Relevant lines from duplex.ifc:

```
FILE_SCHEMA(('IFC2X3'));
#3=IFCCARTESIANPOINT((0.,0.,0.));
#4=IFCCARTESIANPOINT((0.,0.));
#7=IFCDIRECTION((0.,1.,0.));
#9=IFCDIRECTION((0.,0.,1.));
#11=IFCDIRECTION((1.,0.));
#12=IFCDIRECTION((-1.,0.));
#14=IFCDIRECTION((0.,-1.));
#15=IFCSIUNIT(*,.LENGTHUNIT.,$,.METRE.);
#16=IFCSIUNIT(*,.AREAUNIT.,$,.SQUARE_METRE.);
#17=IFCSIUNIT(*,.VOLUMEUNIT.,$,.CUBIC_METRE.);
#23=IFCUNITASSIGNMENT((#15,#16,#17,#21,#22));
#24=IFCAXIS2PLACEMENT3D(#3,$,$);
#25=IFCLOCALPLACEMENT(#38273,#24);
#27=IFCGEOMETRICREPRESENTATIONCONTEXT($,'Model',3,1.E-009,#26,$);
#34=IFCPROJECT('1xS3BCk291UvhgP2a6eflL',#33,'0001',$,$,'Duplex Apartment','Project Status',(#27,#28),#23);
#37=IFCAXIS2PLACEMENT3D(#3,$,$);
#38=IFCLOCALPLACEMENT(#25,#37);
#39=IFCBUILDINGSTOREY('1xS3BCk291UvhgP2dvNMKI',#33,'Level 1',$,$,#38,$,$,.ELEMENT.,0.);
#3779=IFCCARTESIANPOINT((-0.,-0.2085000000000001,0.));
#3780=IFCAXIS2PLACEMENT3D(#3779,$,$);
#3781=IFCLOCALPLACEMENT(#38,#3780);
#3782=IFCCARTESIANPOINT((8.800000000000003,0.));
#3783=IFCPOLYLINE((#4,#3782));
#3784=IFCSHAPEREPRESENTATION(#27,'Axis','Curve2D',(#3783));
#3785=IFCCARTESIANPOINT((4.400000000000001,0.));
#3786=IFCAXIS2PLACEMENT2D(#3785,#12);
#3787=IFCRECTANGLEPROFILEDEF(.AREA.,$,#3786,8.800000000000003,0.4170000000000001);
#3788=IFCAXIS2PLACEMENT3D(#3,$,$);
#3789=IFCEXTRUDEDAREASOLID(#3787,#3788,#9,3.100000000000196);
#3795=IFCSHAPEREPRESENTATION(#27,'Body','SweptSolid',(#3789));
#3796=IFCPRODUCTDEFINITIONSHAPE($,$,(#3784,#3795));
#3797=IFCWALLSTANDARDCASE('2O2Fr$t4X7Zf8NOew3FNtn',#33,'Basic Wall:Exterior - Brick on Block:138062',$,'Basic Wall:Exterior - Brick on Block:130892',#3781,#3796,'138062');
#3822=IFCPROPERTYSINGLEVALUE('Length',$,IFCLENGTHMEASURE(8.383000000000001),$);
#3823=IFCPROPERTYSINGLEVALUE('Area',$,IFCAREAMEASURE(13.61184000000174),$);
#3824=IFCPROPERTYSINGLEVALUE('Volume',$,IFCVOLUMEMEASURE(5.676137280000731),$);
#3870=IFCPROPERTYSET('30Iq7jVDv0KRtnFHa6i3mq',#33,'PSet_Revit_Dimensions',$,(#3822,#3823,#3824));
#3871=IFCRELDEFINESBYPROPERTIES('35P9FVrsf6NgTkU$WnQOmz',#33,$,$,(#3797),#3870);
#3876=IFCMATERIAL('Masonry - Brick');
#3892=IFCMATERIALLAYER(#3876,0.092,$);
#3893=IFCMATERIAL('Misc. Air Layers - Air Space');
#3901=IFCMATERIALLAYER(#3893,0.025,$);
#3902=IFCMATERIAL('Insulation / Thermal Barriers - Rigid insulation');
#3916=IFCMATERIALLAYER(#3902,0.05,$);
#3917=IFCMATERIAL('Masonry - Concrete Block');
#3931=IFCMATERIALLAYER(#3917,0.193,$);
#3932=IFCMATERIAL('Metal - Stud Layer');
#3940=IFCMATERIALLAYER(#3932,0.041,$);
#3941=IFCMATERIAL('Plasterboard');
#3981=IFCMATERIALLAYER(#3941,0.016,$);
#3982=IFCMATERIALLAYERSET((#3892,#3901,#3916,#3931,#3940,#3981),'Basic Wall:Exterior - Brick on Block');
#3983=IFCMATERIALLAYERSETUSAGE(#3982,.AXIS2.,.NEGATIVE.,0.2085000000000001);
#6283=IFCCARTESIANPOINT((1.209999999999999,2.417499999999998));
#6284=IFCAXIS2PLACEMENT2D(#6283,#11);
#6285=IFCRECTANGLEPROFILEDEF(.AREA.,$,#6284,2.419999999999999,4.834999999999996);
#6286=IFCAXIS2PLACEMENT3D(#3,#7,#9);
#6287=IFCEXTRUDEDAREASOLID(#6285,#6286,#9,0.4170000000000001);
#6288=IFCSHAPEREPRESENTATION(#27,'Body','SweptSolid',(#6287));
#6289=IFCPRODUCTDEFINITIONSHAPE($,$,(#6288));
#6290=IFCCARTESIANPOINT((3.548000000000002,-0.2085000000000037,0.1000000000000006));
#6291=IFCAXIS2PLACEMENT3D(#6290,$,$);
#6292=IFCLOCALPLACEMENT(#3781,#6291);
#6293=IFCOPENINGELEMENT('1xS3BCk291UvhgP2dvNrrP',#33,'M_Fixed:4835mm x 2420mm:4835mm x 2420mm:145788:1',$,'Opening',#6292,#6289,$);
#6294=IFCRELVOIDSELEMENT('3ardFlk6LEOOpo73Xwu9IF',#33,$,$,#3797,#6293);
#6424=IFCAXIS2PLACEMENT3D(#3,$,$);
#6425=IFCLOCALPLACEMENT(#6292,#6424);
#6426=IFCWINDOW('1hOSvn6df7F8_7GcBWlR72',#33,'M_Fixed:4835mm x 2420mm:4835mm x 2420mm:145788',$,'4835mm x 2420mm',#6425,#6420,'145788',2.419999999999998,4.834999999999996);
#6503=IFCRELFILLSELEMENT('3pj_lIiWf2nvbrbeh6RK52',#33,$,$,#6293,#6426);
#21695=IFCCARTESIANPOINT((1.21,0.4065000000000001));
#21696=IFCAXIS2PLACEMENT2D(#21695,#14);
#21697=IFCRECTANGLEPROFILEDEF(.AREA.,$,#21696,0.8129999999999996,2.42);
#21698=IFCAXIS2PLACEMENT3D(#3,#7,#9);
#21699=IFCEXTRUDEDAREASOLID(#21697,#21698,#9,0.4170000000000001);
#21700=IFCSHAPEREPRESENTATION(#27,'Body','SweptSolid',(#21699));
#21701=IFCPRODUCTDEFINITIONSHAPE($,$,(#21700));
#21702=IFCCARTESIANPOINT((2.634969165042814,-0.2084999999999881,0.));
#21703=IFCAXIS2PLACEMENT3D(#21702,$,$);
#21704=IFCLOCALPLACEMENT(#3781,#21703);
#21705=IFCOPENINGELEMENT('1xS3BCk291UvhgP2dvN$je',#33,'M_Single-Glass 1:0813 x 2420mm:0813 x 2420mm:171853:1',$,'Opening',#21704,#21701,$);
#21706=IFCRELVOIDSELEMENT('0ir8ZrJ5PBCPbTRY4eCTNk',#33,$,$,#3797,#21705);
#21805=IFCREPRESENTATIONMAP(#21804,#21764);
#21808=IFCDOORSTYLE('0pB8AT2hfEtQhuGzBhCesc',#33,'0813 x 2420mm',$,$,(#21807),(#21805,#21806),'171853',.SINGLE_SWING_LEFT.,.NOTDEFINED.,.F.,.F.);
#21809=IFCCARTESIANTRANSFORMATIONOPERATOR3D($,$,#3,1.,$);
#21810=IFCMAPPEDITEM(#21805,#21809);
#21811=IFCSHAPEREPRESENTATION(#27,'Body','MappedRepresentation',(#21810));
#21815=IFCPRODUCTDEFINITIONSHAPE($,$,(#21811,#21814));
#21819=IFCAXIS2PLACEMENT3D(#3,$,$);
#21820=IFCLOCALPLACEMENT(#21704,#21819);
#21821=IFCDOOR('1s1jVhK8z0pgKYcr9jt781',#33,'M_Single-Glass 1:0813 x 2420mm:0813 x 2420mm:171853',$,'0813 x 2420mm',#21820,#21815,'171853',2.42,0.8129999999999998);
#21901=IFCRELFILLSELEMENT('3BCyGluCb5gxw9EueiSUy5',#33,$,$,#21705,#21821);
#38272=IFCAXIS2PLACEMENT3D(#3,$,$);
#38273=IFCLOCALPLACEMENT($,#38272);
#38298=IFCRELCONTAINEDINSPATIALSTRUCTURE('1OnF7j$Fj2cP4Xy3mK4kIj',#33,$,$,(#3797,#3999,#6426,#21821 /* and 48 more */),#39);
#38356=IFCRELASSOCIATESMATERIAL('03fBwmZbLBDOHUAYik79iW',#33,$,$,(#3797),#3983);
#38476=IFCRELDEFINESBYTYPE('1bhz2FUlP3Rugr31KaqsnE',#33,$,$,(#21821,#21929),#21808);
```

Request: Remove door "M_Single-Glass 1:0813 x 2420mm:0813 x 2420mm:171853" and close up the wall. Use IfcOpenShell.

```python
import ifcopenshell
import ifcopenshell.api.feature
import ifcopenshell.api.pset
import ifcopenshell.api.root
import ifcopenshell.geom
import ifcopenshell.util.element
import ifcopenshell.util.shape
import ifcopenshell.util.unit

model = ifcopenshell.open("duplex.ifc")
area_scale = ifcopenshell.util.unit.calculate_unit_scale(model, "AREAUNIT")
volume_scale = ifcopenshell.util.unit.calculate_unit_scale(model, "VOLUMEUNIT")
settings = ifcopenshell.geom.settings()


def volume(element):
    """Net volume in cubic metres, openings subtracted."""
    shape = ifcopenshell.geom.create_shape(settings, element)
    return ifcopenshell.util.shape.get_volume(shape.geometry)


door = model.by_guid("1s1jVhK8z0pgKYcr9jt781")
opening = door.FillsVoids[0].RelatingOpeningElement
wall = opening.VoidsElements[0].RelatingBuildingElement
before = volume(wall)

ifcopenshell.api.root.remove_product(model, product=door)
ifcopenshell.api.feature.remove_feature(model, feature=opening)

after = volume(wall)
thickness = 0.417  # wall thickness in metres

# Update the wall's stored quantities.
pset = model.by_id(ifcopenshell.util.element.get_pset(wall, "PSet_Revit_Dimensions", should_inherit=False)["id"])
ifcopenshell.api.pset.edit_pset(model, pset=pset, properties={
    "Area": model.create_entity("IfcAreaMeasure", after / thickness / area_scale),
    "Volume": model.create_entity("IfcVolumeMeasure", after / volume_scale),
})

print(f"wall volume {before:.3f} -> {after:.3f} m3")

model.write("duplex_updated.ifc")
```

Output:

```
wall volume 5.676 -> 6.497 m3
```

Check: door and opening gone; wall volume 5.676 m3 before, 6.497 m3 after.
